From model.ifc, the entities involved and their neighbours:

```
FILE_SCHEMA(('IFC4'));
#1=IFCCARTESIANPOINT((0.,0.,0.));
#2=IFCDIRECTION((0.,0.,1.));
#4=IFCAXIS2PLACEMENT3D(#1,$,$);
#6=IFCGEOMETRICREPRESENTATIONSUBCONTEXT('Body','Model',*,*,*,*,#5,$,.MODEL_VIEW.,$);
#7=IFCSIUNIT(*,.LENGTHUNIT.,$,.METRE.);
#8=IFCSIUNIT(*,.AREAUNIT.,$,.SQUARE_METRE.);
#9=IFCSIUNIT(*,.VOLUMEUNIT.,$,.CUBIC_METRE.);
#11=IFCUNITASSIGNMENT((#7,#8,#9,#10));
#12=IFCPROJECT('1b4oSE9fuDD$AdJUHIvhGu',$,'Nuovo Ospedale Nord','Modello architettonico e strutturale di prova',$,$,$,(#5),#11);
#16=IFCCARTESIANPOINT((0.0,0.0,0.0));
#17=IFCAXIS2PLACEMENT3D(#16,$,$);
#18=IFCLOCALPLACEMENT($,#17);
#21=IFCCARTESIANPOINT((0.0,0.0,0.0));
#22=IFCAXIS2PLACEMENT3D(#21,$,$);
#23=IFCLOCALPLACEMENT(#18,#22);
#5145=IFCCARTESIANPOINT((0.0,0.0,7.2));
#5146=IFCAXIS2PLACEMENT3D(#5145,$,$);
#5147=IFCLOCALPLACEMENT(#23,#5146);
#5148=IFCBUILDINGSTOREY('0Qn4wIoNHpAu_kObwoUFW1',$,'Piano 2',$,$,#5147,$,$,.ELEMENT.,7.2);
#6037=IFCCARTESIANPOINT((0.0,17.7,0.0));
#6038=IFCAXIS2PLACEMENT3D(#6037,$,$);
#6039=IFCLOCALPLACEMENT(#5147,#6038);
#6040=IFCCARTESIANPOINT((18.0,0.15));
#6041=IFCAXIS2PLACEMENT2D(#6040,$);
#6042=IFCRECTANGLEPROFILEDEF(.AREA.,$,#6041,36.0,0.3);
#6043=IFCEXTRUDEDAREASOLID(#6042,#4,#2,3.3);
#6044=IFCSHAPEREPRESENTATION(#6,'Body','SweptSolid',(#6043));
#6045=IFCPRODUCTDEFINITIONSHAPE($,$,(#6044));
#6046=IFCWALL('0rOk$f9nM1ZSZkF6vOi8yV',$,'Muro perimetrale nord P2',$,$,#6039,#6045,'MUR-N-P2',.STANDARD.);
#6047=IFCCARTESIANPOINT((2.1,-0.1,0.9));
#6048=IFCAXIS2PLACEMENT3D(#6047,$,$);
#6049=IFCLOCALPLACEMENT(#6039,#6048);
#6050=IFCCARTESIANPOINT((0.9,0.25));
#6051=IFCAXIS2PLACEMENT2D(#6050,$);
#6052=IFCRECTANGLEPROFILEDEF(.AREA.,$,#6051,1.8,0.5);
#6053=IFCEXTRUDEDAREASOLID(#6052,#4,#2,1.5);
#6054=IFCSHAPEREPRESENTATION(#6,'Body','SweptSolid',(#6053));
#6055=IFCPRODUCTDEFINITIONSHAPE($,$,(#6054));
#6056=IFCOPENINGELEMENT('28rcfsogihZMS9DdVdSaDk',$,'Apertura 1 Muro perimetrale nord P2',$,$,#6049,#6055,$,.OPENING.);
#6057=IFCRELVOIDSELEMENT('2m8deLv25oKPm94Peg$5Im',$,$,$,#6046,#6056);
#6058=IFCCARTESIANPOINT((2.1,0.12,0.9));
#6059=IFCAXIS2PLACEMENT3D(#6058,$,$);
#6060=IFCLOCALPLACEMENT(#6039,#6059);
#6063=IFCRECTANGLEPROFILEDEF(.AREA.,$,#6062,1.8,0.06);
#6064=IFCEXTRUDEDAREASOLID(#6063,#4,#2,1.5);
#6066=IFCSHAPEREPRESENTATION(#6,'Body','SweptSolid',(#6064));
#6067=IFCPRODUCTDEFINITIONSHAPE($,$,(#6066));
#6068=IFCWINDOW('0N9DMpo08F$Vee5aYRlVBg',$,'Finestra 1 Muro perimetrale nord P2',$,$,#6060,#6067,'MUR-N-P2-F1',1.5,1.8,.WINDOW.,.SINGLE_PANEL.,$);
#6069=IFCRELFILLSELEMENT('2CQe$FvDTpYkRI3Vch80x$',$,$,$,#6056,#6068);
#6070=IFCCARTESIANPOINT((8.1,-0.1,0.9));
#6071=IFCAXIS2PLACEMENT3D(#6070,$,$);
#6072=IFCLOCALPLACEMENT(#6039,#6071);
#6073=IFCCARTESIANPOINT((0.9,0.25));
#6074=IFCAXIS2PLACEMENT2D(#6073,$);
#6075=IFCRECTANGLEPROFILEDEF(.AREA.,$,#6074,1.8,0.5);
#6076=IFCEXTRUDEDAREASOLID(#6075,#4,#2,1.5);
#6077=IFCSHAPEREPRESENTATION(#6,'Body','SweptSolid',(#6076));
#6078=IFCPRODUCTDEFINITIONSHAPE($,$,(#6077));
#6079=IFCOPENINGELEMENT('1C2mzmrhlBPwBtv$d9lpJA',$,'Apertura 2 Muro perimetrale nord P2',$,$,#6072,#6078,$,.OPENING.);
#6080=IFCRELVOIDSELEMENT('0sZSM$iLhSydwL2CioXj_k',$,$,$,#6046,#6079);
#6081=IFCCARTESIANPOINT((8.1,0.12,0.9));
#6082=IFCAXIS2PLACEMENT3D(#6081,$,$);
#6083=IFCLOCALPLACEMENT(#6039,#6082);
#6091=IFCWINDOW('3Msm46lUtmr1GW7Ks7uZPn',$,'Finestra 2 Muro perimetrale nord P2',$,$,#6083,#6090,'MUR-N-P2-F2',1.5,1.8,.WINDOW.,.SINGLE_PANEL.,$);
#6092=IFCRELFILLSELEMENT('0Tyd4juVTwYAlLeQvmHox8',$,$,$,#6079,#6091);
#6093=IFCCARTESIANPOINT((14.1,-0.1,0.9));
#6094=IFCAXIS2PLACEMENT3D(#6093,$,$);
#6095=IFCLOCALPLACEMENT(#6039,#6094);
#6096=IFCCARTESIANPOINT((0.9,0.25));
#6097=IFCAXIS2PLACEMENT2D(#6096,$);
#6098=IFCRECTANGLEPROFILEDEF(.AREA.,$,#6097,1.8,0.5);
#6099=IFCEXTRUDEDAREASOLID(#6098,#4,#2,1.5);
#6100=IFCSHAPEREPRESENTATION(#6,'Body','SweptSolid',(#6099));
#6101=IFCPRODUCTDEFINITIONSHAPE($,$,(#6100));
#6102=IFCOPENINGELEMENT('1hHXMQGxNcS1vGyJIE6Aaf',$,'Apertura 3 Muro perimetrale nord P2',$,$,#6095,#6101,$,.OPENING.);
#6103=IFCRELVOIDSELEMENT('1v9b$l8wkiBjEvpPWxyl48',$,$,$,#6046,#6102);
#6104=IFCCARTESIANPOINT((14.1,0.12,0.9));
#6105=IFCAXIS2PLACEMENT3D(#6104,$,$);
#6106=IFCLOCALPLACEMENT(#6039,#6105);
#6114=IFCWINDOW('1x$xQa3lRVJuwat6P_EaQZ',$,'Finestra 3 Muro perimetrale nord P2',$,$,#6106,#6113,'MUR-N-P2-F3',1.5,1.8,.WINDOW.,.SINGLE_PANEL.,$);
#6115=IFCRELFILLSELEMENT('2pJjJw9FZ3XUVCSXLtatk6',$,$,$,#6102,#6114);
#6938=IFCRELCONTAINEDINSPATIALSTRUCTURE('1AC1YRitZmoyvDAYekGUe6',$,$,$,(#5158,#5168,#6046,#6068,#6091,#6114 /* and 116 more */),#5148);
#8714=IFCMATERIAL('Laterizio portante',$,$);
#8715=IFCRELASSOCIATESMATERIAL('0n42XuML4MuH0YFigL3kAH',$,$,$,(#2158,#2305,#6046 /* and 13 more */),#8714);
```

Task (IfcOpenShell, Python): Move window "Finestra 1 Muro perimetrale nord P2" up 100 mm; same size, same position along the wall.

```python
import numpy as np
import ifcopenshell
import ifcopenshell.api.geometry
import ifcopenshell.util.placement
import ifcopenshell.util.unit

model = ifcopenshell.open("model.ifc")
unit_scale = ifcopenshell.util.unit.calculate_unit_scale(model)

window = model.by_guid("0N9DMpo08F$Vee5aYRlVBg")
opening = window.FillsVoids[0].RelatingOpeningElement
dz = 0.1 / unit_scale

shift = np.array([0.0, 0.0, dz])
# The window is not placed relative to its opening, so move both.
for product in (opening, window):
    matrix = ifcopenshell.util.placement.get_local_placement(product.ObjectPlacement)
    matrix[:3, 3] += shift
    ifcopenshell.api.geometry.edit_object_placement(model, product=product, matrix=matrix, is_si=False)

print(f"moved by {dz * unit_scale:+.3f} m")

model.write("model_updated.ifc")
```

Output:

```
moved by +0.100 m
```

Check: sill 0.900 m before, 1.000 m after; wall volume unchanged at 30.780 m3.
